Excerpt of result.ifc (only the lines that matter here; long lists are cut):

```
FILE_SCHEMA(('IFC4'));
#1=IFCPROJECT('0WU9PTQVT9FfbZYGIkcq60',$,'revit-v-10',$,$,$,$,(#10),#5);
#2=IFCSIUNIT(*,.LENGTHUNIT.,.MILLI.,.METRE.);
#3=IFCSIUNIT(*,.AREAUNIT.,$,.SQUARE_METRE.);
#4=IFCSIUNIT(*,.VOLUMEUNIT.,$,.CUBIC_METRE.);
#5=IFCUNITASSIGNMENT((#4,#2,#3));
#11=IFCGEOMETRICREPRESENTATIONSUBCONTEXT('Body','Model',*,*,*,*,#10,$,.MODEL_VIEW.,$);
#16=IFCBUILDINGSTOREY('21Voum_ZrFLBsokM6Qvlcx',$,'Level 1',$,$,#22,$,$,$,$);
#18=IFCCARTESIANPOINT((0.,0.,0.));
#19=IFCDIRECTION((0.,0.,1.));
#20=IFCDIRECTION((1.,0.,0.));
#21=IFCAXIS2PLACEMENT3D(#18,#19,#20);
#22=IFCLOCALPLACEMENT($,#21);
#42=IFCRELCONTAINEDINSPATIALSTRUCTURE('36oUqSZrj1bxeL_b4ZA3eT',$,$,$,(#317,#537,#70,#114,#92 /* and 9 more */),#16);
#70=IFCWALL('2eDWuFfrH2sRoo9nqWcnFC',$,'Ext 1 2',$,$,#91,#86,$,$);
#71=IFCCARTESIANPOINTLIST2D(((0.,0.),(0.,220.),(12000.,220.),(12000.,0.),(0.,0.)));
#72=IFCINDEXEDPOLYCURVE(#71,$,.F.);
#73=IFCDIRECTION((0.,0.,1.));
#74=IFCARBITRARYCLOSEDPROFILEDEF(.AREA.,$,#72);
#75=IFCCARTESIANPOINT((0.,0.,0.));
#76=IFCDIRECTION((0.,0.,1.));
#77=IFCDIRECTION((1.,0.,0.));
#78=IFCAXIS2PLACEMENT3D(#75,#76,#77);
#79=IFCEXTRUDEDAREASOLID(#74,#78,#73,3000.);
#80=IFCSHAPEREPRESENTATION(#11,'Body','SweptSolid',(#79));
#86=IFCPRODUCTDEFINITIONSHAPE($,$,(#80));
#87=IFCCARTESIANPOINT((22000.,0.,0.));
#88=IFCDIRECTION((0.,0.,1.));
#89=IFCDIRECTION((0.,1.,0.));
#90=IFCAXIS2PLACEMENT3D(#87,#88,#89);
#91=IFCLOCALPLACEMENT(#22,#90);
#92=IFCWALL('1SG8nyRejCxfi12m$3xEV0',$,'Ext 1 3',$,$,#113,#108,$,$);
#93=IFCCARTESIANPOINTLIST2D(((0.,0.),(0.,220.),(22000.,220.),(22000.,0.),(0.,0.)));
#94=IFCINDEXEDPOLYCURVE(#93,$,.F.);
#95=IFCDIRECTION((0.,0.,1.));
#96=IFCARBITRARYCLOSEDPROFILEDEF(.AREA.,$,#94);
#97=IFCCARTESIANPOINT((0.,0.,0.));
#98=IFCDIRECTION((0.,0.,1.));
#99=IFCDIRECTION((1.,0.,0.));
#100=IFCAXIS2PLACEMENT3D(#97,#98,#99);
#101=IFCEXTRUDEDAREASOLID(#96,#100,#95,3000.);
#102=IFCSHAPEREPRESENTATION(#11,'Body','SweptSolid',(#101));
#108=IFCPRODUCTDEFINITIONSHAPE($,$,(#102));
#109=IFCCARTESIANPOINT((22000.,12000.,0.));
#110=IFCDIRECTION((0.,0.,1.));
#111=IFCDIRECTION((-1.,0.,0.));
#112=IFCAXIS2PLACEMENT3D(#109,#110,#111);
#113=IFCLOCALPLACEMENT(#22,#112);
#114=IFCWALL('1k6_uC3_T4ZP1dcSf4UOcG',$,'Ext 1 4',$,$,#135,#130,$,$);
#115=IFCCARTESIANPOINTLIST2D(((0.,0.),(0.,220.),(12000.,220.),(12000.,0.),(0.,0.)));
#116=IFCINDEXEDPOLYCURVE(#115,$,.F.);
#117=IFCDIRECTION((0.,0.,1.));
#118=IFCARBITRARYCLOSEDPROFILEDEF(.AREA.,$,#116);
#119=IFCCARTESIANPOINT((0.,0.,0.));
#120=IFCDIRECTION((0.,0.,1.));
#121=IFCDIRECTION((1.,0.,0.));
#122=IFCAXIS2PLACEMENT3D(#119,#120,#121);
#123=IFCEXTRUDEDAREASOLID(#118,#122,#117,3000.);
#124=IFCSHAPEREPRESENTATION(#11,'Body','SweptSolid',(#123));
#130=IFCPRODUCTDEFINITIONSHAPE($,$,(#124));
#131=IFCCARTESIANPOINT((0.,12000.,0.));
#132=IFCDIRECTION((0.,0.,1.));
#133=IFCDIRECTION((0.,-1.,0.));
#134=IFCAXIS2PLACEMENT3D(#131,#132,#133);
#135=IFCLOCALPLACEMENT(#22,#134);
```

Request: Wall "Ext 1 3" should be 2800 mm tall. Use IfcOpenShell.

```python
import ifcopenshell
import ifcopenshell.geom
import ifcopenshell.util.representation
import ifcopenshell.util.shape
import ifcopenshell.util.unit

model = ifcopenshell.open("result.ifc")
unit_scale = ifcopenshell.util.unit.calculate_unit_scale(model)
settings = ifcopenshell.geom.settings()


def volume(element):
    """Net volume in cubic metres, openings subtracted."""
    shape = ifcopenshell.geom.create_shape(settings, element)
    return ifcopenshell.util.shape.get_volume(shape.geometry)


wall = model.by_id(92)
before = volume(wall)

body = ifcopenshell.util.representation.get_representation(wall, "Model", "Body")
solid = body.Items[0]
old_height = solid.Depth
solid.Depth = 2.8 / unit_scale
after = volume(wall)

print(f"height {old_height:g} -> {solid.Depth:g}, volume {before:.3f} -> {after:.3f} m3")

model.write("result_updated.ifc")
```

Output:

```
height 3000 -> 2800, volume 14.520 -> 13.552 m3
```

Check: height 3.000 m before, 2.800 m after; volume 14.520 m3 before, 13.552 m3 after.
